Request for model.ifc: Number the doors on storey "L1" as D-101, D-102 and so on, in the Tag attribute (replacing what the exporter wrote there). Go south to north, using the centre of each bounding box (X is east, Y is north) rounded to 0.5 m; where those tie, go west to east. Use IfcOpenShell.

First a look at what the model holds.

```python
import ifcopenshell
import ifcopenshell.util.element
import ifcopenshell.util.placement

model = ifcopenshell.open("model.ifc")
print(model.schema)
storey = next(s for s in model.by_type("IfcBuildingStorey") if s.Name == "L1")
doors = [e for e in ifcopenshell.util.element.get_decomposition(storey) if e.is_a("IfcDoor")]
for e in sorted(doors, key=lambda e: e.id()):
    origin = ifcopenshell.util.placement.get_local_placement(e.ObjectPlacement)[:3, 3]
    print(e.id(), e.Tag, e.Name, origin.round(2) + 0.0, sep=" | ")
```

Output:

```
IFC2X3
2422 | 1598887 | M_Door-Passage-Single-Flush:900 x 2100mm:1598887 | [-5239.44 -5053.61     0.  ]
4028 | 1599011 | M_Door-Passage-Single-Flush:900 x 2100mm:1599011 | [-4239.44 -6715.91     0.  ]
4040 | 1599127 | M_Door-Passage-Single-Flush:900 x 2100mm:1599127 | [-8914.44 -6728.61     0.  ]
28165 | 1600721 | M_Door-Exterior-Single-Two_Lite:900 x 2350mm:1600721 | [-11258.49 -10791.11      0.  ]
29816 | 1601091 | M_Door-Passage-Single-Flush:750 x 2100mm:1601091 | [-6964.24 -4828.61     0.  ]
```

```python
import ifcopenshell
import ifcopenshell.geom
import ifcopenshell.util.element
import ifcopenshell.util.shape

model = ifcopenshell.open("model.ifc")
settings = ifcopenshell.geom.settings()
settings.set("use-world-coords", True)


def centre(element):
    shape = ifcopenshell.geom.create_shape(settings, element)
    return ifcopenshell.util.shape.get_bbox_centroid(shape.geometry)


storey = next(s for s in model.by_type("IfcBuildingStorey") if s.Name == "L1")
doors = [e for e in ifcopenshell.util.element.get_decomposition(storey) if e.is_a("IfcDoor")]

# Insertion points can sit at a corner or the storey origin, so sort by the geometry (in metres).
centres = {e: centre(e) for e in doors}
doors.sort(key=lambda e: (round(centres[e][1] / 0.5), centres[e][0]))

for i, e in enumerate(doors, start=1):
    number = f"D-1{i:02d}"
    e.Tag = number
    print(e.id(), number)

model.write("model_updated.ifc")
```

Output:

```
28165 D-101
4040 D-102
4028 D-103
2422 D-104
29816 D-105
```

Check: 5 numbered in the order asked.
